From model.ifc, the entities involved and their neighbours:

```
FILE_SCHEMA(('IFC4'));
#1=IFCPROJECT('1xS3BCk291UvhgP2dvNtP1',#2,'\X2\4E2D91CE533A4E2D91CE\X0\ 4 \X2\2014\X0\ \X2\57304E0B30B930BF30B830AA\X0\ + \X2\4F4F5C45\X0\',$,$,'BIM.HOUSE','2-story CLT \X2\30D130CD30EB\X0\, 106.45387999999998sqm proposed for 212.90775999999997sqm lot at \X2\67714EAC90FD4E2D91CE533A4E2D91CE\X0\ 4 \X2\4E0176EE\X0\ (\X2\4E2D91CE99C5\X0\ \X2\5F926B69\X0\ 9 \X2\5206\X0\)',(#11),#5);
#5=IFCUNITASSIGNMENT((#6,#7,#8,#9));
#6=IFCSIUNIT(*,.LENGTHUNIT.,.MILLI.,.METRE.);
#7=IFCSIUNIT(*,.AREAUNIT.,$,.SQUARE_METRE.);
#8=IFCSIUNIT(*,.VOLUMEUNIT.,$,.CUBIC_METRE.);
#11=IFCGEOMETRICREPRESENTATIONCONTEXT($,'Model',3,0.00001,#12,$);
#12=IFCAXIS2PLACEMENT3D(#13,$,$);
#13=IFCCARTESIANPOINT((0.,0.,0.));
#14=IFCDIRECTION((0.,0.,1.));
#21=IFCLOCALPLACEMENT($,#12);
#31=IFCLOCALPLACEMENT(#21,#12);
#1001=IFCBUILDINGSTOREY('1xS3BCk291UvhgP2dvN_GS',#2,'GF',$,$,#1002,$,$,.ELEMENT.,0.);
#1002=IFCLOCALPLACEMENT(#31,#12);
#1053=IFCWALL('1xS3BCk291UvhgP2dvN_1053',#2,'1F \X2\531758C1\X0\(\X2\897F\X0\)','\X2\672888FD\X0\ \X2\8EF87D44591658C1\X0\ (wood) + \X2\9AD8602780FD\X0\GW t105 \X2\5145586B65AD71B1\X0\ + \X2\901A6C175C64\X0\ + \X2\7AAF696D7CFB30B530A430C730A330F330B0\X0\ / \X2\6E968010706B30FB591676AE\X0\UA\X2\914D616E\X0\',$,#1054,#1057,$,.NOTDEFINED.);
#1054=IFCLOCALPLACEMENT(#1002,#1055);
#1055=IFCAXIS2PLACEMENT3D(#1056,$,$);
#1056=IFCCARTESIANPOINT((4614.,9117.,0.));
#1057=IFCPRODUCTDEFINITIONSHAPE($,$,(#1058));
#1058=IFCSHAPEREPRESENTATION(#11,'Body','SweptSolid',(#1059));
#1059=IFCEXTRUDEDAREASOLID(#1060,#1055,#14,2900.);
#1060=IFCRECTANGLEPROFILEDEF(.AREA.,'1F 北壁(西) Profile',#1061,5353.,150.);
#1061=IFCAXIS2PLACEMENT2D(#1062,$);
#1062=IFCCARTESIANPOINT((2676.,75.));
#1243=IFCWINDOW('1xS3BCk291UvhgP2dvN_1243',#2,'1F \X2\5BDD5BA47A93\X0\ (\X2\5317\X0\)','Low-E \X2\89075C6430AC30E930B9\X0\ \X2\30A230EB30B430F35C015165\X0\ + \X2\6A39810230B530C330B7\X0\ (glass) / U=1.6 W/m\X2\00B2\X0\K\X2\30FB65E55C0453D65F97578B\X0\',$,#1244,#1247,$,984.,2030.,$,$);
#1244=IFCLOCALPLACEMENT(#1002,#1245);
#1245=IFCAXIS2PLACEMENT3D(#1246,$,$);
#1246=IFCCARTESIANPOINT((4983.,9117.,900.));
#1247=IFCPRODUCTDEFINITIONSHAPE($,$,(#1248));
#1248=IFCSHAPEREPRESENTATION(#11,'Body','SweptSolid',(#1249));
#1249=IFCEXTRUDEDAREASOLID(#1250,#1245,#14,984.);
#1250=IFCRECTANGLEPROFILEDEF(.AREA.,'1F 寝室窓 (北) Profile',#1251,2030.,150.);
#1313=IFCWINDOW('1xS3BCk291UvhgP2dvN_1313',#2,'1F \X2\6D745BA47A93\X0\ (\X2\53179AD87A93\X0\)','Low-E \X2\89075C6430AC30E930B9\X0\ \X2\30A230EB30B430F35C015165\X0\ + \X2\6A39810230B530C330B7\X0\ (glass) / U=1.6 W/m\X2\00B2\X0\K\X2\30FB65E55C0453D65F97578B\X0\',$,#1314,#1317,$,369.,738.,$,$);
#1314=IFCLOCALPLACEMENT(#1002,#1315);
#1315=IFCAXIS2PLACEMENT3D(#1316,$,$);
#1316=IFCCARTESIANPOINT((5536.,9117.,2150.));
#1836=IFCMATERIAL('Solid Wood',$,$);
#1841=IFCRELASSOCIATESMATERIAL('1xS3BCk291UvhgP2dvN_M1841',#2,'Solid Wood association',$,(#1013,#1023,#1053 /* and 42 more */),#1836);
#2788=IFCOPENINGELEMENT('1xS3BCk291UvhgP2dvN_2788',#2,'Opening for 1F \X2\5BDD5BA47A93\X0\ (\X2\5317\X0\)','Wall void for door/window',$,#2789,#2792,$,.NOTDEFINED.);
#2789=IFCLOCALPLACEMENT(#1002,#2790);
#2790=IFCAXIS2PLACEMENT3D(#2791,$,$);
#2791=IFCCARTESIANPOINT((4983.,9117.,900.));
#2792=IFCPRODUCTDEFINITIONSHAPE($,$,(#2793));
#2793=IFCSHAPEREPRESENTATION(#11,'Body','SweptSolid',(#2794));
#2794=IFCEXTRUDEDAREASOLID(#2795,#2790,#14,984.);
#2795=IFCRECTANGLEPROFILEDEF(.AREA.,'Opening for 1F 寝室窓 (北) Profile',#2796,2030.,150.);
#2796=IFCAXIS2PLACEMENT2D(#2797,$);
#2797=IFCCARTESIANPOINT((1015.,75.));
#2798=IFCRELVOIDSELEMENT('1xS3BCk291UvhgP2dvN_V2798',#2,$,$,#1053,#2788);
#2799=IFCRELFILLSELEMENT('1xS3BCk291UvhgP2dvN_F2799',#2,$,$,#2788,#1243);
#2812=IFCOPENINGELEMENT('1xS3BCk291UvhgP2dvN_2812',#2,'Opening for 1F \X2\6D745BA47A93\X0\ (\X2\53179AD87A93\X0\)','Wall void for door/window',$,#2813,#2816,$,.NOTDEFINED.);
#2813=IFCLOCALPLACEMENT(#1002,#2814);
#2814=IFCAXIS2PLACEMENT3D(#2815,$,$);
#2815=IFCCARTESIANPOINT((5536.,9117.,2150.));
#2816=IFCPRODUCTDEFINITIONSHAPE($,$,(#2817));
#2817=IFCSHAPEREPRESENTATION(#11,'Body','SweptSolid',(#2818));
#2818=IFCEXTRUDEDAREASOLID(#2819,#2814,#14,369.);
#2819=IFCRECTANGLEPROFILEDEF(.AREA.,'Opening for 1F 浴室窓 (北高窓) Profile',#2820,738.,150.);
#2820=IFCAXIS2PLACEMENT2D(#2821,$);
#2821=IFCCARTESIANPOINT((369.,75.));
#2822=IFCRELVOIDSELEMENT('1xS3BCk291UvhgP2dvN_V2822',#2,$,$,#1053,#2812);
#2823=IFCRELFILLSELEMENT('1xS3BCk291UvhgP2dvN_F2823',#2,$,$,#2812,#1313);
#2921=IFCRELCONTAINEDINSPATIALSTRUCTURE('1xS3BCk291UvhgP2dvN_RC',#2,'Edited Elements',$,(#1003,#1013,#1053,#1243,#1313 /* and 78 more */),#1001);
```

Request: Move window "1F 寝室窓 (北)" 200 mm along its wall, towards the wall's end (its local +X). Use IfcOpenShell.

```python
import ifcopenshell
import ifcopenshell.api.geometry
import ifcopenshell.util.placement
import ifcopenshell.util.unit

model = ifcopenshell.open("model.ifc")
unit_scale = ifcopenshell.util.unit.calculate_unit_scale(model)

window = model.by_guid("1xS3BCk291UvhgP2dvN_1243")
opening = window.FillsVoids[0].RelatingOpeningElement
wall = opening.VoidsElements[0].RelatingBuildingElement

wall_matrix = ifcopenshell.util.placement.get_local_placement(wall.ObjectPlacement)
shift = wall_matrix[:3, 0] * 0.2 / unit_scale
before = ifcopenshell.util.placement.get_local_placement(window.ObjectPlacement)[:3, 3].copy()

# The window is not placed relative to its opening, so move both.
for product in (opening, window):
    matrix = ifcopenshell.util.placement.get_local_placement(product.ObjectPlacement)
    matrix[:3, 3] += shift
    ifcopenshell.api.geometry.edit_object_placement(model, product=product, matrix=matrix, is_si=False)

after = ifcopenshell.util.placement.get_local_placement(window.ObjectPlacement)[:3, 3]
print("window moved by", (after - before).round(3) + 0.0)

model.write("model_updated.ifc")
```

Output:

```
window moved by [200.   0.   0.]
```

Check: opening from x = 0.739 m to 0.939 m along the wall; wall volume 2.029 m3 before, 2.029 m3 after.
